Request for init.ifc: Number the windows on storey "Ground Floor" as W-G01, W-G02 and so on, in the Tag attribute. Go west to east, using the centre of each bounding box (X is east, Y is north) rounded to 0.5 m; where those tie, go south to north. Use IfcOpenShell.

First a look at what the model holds.

```python
import ifcopenshell
import ifcopenshell.util.element
import ifcopenshell.util.placement

model = ifcopenshell.open("init.ifc")
print(model.schema)
storey = next(s for s in model.by_type("IfcBuildingStorey") if s.Name == "Ground Floor")
windows = [e for e in ifcopenshell.util.element.get_decomposition(storey) if e.is_a("IfcWindow")]
for e in sorted(windows, key=lambda e: e.id()):
    origin = ifcopenshell.util.placement.get_local_placement(e.ObjectPlacement)[:3, 3]
    print(e.id(), e.Tag, e.Name, origin.round(2) + 0.0, sep=" | ")
```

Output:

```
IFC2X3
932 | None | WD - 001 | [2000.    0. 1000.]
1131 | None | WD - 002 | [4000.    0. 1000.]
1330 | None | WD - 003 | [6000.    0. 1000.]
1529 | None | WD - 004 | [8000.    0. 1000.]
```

```python
import ifcopenshell
import ifcopenshell.geom
import ifcopenshell.util.element
import ifcopenshell.util.shape

model = ifcopenshell.open("init.ifc")
settings = ifcopenshell.geom.settings()
settings.set("use-world-coords", True)


def centre(element):
    shape = ifcopenshell.geom.create_shape(settings, element)
    return ifcopenshell.util.shape.get_bbox_centroid(shape.geometry)


storey = next(s for s in model.by_type("IfcBuildingStorey") if s.Name == "Ground Floor")
windows = [e for e in ifcopenshell.util.element.get_decomposition(storey) if e.is_a("IfcWindow")]

# Insertion points can sit at a corner or the storey origin, so sort by the geometry (in metres).
centres = {e: centre(e) for e in windows}
windows.sort(key=lambda e: (round(centres[e][0] / 0.5), centres[e][1]))

for i, e in enumerate(windows, start=1):
    number = f"W-G{i:02d}"
    e.Tag = number
    print(e.id(), number)

model.write("init_edited.ifc")
```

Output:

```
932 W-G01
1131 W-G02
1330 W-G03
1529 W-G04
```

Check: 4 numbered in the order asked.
